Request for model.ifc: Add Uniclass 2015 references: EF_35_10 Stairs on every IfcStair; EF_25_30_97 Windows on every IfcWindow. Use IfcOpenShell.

First a look at what the model holds.

```python
import ifcopenshell

model = ifcopenshell.open("model.ifc")
print(model.schema)
print("classifications:", [c.Name for c in model.by_type("IfcClassification")])
for ifc_class in ("IfcDoor", "IfcRoof", "IfcStair", "IfcWall", "IfcWindow"):
    print(ifc_class, len(model.by_type(ifc_class)))
```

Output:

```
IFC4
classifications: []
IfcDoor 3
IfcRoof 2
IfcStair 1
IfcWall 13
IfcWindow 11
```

```python
import ifcopenshell
import ifcopenshell.api.classification

model = ifcopenshell.open("model.ifc")

system = ifcopenshell.api.classification.add_classification(model, classification="Uniclass 2015")

codes = {
    "IfcStair": ("EF_35_10", "Stairs"),
    "IfcWindow": ("EF_25_30_97", "Windows"),
}
for ifc_class, (code, name) in codes.items():
    products = model.by_type(ifc_class)
    ifcopenshell.api.classification.add_reference(
        model, products=products, classification=system, identification=code, name=name
    )
    print(code, len(products))

model.write("model_v2.ifc")
```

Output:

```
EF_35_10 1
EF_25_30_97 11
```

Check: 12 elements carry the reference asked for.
